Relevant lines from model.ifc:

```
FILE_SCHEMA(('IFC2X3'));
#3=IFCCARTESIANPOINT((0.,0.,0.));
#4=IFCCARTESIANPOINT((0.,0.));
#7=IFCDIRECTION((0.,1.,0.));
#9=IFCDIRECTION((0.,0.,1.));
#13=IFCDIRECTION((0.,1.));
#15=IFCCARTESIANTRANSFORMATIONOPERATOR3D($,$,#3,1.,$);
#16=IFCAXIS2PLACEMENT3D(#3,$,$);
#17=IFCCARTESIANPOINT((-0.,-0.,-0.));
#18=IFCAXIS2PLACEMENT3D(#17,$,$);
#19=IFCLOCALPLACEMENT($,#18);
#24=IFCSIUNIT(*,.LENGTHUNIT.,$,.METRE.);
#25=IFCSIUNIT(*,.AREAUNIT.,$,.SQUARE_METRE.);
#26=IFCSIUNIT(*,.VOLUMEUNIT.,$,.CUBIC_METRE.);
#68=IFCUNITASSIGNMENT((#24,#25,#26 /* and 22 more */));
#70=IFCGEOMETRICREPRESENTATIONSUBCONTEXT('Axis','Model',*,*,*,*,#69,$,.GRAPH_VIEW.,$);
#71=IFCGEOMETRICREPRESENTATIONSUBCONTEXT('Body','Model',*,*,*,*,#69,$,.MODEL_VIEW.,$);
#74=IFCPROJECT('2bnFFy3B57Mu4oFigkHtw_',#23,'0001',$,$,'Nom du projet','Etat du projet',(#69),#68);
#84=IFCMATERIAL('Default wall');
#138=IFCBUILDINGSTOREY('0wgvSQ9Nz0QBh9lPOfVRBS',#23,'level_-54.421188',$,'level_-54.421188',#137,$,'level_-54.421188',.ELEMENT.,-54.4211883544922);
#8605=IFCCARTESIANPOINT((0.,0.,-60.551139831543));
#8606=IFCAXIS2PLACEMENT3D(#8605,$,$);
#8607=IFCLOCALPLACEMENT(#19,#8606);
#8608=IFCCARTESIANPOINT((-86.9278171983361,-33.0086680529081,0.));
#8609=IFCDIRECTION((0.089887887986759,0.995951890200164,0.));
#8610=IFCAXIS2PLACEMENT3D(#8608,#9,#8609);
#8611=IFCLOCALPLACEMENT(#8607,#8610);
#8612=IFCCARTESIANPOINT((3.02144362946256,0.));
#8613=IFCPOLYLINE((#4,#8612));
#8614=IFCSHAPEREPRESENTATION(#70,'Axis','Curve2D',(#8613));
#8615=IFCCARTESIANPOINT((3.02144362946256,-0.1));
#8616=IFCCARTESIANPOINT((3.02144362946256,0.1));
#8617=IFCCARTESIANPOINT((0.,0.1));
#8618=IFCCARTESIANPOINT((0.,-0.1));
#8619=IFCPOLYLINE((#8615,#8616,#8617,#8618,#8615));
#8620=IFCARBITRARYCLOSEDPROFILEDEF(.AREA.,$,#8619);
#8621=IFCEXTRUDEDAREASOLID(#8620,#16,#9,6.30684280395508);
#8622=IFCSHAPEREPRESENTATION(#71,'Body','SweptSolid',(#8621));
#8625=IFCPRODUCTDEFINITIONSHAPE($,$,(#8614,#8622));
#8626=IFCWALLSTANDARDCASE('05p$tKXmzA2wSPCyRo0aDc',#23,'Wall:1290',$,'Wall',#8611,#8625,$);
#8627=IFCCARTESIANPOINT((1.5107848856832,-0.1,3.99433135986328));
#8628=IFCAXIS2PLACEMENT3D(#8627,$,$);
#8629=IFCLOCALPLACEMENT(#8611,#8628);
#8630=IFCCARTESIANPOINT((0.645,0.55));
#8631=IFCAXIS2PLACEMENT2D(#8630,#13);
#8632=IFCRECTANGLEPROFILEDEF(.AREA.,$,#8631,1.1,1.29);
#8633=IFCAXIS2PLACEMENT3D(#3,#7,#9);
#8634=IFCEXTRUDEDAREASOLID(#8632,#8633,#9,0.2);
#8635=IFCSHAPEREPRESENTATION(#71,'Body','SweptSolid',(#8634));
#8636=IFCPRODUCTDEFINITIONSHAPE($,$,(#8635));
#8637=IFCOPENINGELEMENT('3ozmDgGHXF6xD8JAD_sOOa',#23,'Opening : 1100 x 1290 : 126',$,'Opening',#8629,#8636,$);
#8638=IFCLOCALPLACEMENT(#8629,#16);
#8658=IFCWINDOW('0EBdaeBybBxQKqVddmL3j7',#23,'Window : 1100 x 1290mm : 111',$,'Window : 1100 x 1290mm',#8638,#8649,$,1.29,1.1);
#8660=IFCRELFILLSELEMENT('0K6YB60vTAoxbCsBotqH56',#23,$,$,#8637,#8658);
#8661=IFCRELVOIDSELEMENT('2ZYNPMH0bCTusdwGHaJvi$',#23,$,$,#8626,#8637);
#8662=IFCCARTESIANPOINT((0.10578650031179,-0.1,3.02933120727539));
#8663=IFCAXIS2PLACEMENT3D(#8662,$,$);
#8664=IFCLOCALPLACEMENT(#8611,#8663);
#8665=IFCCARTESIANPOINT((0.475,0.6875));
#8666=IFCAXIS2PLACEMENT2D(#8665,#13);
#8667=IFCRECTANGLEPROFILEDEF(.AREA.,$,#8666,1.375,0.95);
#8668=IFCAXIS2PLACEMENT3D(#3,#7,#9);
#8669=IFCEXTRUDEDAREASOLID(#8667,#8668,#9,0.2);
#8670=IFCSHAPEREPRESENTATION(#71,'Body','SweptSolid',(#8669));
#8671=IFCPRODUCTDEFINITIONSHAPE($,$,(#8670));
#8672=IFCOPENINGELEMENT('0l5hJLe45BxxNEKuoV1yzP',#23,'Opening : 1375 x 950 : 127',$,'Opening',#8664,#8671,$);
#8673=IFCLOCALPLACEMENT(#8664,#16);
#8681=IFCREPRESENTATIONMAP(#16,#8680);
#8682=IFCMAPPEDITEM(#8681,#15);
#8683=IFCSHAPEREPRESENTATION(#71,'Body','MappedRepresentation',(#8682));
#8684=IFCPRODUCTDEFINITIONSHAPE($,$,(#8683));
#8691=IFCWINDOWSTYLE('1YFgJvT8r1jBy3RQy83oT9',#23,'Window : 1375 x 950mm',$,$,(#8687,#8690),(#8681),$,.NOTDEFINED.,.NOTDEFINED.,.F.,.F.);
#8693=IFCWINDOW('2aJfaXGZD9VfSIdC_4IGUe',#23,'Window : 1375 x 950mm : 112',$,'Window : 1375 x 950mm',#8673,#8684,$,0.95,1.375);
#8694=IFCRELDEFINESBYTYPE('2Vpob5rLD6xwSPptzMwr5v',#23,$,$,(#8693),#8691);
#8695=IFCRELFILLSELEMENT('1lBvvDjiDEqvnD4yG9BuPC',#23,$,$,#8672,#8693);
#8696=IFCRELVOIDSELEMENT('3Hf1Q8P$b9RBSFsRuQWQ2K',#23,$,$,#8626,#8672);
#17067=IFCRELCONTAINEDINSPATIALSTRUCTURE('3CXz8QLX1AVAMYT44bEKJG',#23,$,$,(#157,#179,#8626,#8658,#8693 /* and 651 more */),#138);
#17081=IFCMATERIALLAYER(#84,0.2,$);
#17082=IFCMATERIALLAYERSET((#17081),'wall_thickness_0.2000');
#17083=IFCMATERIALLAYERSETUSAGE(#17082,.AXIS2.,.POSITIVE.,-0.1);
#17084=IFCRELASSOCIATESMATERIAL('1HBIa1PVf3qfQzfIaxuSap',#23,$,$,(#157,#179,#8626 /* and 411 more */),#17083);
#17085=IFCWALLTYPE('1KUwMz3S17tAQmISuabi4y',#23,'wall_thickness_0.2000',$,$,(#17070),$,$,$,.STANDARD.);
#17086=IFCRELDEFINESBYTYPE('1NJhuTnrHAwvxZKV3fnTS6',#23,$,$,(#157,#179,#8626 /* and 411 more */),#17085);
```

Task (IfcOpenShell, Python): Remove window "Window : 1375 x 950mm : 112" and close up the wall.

```python
import ifcopenshell
import ifcopenshell.api.feature
import ifcopenshell.api.root
import ifcopenshell.geom
import ifcopenshell.util.shape

model = ifcopenshell.open("model.ifc")
settings = ifcopenshell.geom.settings()


def volume(element):
    """Net volume in cubic metres, openings subtracted."""
    shape = ifcopenshell.geom.create_shape(settings, element)
    return ifcopenshell.util.shape.get_volume(shape.geometry)


window = model.by_id(8693)
opening = window.FillsVoids[0].RelatingOpeningElement
wall = opening.VoidsElements[0].RelatingBuildingElement
before = volume(wall)

ifcopenshell.api.root.remove_product(model, product=window)
ifcopenshell.api.feature.remove_feature(model, feature=opening)

after = volume(wall)

print(f"wall volume {before:.3f} -> {after:.3f} m3")

model.write("model_rev.ifc")
```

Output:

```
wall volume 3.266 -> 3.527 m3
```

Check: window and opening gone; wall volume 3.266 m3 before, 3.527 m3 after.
